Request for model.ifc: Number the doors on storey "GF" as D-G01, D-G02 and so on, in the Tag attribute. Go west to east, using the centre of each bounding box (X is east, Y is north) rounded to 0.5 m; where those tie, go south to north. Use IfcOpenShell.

First a look at what the model holds.

```python
import ifcopenshell
import ifcopenshell.util.element
import ifcopenshell.util.placement

model = ifcopenshell.open("model.ifc")
print(model.schema)
storey = next(s for s in model.by_type("IfcBuildingStorey") if s.Name == "GF")
doors = [e for e in ifcopenshell.util.element.get_decomposition(storey) if e.is_a("IfcDoor")]
for e in sorted(doors, key=lambda e: e.id()):
    origin = ifcopenshell.util.placement.get_local_placement(e.ObjectPlacement)[:3, 3]
    print(e.id(), e.Tag, e.Name, origin.round(2) + 0.0, sep=" | ")
```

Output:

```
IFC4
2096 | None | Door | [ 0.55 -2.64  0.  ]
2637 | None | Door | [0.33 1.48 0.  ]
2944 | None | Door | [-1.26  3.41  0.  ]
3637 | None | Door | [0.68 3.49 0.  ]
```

```python
import ifcopenshell
import ifcopenshell.geom
import ifcopenshell.util.element
import ifcopenshell.util.shape

model = ifcopenshell.open("model.ifc")
settings = ifcopenshell.geom.settings()
settings.set("use-world-coords", True)


def centre(element):
    shape = ifcopenshell.geom.create_shape(settings, element)
    return ifcopenshell.util.shape.get_bbox_centroid(shape.geometry)


storey = next(s for s in model.by_type("IfcBuildingStorey") if s.Name == "GF")
doors = [e for e in ifcopenshell.util.element.get_decomposition(storey) if e.is_a("IfcDoor")]

# Insertion points can sit at a corner or the storey origin, so sort by the geometry (in metres).
centres = {e: centre(e) for e in doors}
doors.sort(key=lambda e: (round(centres[e][0] / 0.5), centres[e][1]))

for i, e in enumerate(doors, start=1):
    number = f"D-G{i:02d}"
    e.Tag = number
    print(e.id(), number)

model.write("model_updated.ifc")
```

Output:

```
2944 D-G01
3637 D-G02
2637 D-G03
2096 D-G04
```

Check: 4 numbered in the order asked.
